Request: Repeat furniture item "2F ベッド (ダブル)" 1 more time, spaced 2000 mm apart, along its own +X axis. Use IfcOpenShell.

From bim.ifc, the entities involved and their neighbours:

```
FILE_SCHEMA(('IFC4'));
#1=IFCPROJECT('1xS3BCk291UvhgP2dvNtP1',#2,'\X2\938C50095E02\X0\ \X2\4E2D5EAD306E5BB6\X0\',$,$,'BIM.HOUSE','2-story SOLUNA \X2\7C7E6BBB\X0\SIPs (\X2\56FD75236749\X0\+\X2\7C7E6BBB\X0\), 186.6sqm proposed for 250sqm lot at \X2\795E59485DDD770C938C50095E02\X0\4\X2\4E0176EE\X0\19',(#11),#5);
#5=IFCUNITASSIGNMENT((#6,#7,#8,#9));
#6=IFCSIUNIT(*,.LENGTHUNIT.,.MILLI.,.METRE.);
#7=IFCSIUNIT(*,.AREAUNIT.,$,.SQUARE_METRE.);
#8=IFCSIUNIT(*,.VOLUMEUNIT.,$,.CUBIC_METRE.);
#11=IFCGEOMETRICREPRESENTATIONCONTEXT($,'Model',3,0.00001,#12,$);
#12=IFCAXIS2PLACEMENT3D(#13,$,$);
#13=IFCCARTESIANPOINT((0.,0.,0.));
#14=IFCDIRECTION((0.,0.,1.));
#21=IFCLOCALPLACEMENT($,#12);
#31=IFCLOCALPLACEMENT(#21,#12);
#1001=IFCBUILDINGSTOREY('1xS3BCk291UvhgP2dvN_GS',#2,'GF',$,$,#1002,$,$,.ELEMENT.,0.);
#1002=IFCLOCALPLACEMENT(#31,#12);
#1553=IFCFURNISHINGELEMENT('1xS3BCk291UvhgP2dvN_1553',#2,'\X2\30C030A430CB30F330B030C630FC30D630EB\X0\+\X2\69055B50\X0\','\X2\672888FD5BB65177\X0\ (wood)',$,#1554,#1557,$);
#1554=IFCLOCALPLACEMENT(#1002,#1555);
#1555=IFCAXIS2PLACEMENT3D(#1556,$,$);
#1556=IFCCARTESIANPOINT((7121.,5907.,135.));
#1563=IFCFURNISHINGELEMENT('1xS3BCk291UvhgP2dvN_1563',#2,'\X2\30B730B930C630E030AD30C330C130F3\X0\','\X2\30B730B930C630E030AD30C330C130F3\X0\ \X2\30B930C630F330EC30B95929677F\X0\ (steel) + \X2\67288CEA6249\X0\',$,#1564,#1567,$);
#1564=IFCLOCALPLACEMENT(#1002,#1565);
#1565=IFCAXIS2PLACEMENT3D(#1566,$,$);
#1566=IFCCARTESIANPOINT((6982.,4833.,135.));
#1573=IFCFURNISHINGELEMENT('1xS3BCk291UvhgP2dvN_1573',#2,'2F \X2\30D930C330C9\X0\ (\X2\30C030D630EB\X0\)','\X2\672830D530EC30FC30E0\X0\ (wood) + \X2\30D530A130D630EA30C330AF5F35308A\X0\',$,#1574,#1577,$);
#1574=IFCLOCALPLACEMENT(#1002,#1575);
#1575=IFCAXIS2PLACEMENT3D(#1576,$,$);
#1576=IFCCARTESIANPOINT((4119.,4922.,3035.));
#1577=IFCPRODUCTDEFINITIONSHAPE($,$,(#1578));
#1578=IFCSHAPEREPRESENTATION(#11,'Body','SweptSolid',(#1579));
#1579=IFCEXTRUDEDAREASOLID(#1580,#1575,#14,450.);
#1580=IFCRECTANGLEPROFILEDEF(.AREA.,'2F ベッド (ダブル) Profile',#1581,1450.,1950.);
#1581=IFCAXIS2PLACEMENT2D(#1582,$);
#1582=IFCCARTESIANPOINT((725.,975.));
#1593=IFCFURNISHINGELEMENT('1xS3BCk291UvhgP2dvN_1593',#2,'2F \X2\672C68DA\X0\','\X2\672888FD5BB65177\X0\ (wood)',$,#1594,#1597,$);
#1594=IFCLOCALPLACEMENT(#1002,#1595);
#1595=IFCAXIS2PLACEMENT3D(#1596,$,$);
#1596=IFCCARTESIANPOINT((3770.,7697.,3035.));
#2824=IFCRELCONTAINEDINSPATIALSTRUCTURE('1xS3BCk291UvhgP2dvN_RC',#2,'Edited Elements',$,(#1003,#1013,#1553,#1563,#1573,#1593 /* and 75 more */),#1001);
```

```python
import ifcopenshell
import ifcopenshell.api.geometry
import ifcopenshell.api.root
import ifcopenshell.util.element
import ifcopenshell.util.placement
import ifcopenshell.util.unit

model = ifcopenshell.open("bim.ifc")
unit_scale = ifcopenshell.util.unit.calculate_unit_scale(model)


def reuse_history(source, copy):
    """copy_class also copies each property set's owner history, people and application; keep the originals."""
    for rel in copy.IsDefinedBy:
        if rel.is_a("IfcRelDefinesByProperties") and (history := rel.RelatingPropertyDefinition.OwnerHistory):
            rel.RelatingPropertyDefinition.OwnerHistory = source.OwnerHistory
            ifcopenshell.util.element.remove_deep2(model, history)


source = model.by_guid("1xS3BCk291UvhgP2dvN_1573")
base = ifcopenshell.util.placement.get_local_placement(source.ObjectPlacement)
step = base[:3, 0] * 2 / unit_scale

for i in range(1, 2):
    copy = ifcopenshell.api.root.copy_class(model, product=source)
    copy.Representation = ifcopenshell.util.element.copy_deep(
        model, source.Representation, exclude=["IfcGeometricRepresentationContext", "IfcRepresentationMap"]
    )
    reuse_history(source, copy)
    matrix = base.copy()
    matrix[:3, 3] += i * step
    print("added at", matrix[:3, 3].round(3) + 0.0)
    ifcopenshell.api.geometry.edit_object_placement(model, product=copy, matrix=matrix, is_si=False)

model.write("bim_edited.ifc")
```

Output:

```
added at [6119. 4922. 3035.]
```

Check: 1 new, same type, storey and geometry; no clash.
